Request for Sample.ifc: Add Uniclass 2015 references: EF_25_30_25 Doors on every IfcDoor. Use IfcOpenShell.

First a look at what the model holds.

```python
import ifcopenshell

model = ifcopenshell.open("Sample.ifc")
print(model.schema)
print("classifications:", [c.Name for c in model.by_type("IfcClassification")])
for ifc_class in ("IfcDoor", "IfcRoof", "IfcStair", "IfcWall", "IfcWindow"):
    print(ifc_class, len(model.by_type(ifc_class)))
```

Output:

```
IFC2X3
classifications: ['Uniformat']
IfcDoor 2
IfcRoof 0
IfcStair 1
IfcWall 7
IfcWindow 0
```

```python
import ifcopenshell
import ifcopenshell.api.classification

model = ifcopenshell.open("Sample.ifc")

# IFC2X3 requires Source and Edition and has no link from the project to the system.
system = model.create_entity("IfcClassification", Source="NBS", Edition="2015", Name="Uniclass 2015")

codes = {
    "IfcDoor": ("EF_25_30_25", "Doors"),
}
for ifc_class, (code, name) in codes.items():
    products = model.by_type(ifc_class)
    ifcopenshell.api.classification.add_reference(
        model, products=products, classification=system, identification=code, name=name
    )
    print(code, len(products))

model.write("Sample-out.ifc")
```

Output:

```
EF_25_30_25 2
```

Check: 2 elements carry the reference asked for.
